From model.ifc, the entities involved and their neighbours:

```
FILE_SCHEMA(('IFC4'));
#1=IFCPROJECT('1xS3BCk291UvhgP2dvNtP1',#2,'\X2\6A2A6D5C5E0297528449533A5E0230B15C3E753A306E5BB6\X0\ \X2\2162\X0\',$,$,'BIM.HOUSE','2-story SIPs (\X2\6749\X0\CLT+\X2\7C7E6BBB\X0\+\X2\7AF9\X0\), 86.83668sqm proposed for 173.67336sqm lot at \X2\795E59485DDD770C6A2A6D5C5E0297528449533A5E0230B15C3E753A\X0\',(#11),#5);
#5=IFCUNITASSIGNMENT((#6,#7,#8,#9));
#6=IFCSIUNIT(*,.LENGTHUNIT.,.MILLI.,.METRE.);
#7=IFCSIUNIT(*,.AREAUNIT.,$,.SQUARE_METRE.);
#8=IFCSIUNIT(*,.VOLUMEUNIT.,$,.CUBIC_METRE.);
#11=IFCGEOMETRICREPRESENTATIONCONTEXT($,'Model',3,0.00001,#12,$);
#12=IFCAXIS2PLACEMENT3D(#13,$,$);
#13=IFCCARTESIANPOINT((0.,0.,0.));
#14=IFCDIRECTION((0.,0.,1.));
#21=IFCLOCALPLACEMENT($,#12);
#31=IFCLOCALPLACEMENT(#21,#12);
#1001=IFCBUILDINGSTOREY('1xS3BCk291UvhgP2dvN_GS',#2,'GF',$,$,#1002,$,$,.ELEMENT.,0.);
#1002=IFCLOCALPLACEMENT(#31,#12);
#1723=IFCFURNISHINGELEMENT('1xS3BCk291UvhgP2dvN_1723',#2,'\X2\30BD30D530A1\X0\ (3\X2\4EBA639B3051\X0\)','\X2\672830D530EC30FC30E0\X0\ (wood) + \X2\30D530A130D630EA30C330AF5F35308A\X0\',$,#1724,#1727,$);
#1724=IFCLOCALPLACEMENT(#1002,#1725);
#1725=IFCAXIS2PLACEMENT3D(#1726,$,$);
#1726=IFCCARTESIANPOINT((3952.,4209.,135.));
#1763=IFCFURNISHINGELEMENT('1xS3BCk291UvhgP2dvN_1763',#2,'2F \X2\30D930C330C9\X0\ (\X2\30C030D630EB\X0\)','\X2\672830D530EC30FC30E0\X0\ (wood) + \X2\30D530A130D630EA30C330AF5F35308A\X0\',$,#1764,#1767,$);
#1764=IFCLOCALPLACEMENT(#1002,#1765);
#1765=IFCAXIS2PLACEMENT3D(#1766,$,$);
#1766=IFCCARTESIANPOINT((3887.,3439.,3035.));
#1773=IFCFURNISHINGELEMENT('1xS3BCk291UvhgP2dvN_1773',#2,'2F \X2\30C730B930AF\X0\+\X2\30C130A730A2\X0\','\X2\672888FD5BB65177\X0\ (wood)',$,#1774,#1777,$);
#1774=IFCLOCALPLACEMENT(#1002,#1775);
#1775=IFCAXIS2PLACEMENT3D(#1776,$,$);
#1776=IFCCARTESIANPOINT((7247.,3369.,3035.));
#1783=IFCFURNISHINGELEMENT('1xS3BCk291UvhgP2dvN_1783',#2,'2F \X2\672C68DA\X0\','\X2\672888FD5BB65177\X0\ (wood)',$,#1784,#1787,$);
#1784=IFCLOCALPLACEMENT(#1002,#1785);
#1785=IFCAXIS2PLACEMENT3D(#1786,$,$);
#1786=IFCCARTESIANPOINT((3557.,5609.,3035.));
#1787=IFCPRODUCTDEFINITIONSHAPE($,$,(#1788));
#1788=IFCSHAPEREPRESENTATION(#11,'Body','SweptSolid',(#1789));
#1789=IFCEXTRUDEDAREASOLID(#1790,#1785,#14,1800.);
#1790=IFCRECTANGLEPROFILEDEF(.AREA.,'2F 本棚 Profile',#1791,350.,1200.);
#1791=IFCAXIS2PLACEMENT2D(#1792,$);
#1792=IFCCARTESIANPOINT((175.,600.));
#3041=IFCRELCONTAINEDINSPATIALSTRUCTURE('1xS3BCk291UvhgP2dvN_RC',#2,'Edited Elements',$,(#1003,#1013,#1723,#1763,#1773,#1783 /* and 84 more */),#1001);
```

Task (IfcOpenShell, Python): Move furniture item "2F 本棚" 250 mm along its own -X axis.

```python
import ifcopenshell
import ifcopenshell.api.geometry
import ifcopenshell.util.placement

model = ifcopenshell.open("model.ifc")

item = model.by_id(1783)
matrix = ifcopenshell.util.placement.get_local_placement(item.ObjectPlacement)
matrix[:3, 3] -= matrix[:3, 0] * 250.0
ifcopenshell.api.geometry.edit_object_placement(model, product=item, matrix=matrix, is_si=False)

print(ifcopenshell.util.placement.get_local_placement(item.ObjectPlacement).round(3) + 0.0)

model.write("model_edited.ifc")
```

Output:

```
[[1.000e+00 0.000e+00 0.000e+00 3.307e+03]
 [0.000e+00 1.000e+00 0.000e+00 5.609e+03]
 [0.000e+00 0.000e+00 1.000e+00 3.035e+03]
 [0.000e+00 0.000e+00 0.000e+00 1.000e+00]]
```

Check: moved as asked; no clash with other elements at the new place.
